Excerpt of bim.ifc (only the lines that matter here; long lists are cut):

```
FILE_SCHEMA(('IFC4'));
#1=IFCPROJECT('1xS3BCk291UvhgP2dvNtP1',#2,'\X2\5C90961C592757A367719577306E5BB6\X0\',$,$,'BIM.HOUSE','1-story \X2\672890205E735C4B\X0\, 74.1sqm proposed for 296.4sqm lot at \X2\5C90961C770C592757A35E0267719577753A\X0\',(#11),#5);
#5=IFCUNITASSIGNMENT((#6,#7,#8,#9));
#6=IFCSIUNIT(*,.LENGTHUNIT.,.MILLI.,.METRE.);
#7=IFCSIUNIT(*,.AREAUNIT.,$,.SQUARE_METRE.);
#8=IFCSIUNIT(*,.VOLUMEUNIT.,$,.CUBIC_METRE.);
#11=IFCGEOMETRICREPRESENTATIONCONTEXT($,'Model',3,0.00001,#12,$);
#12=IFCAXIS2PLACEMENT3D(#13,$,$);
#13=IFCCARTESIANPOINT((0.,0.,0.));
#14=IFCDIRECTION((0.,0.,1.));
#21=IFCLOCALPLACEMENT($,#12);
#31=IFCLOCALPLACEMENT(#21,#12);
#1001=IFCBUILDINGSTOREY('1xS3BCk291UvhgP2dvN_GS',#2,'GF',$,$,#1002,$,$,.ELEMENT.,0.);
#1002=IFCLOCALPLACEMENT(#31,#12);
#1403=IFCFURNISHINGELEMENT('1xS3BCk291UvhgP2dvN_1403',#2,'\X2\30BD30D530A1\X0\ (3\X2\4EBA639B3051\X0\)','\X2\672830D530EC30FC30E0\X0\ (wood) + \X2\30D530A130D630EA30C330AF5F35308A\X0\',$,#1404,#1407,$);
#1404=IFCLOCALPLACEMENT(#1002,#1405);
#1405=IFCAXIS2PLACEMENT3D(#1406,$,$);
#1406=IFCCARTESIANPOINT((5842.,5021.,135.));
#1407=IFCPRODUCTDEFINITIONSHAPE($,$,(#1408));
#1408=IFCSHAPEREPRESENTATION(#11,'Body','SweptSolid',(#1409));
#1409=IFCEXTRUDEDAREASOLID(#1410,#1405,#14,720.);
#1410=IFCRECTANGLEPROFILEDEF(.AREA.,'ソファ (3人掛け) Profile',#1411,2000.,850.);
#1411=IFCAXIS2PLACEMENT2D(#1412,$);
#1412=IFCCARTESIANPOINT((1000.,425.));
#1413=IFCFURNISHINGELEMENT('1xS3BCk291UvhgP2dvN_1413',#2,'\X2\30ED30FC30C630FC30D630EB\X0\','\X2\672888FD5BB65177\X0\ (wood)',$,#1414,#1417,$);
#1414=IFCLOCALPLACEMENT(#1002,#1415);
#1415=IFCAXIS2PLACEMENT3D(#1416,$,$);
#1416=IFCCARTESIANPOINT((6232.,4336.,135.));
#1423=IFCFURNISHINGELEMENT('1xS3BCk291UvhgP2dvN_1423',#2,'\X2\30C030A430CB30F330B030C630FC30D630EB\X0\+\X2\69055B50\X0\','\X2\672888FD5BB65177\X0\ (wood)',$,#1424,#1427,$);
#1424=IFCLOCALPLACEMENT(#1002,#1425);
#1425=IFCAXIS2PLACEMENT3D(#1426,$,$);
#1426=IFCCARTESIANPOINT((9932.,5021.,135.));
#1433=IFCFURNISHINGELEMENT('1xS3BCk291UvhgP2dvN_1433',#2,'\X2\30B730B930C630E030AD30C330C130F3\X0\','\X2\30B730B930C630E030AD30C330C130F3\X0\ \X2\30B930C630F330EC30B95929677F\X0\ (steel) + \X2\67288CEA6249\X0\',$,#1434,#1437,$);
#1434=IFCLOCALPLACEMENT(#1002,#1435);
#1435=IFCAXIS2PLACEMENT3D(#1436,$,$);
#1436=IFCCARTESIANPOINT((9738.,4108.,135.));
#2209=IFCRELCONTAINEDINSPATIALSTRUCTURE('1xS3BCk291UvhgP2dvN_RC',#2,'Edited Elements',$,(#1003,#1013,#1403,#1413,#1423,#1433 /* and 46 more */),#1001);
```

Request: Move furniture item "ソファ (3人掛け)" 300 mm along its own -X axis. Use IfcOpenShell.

```python
import ifcopenshell
import ifcopenshell.api.geometry
import ifcopenshell.util.placement
import ifcopenshell.util.unit

model = ifcopenshell.open("bim.ifc")
unit_scale = ifcopenshell.util.unit.calculate_unit_scale(model)

item = model.by_guid("1xS3BCk291UvhgP2dvN_1403")
matrix = ifcopenshell.util.placement.get_local_placement(item.ObjectPlacement)
matrix[:3, 3] -= matrix[:3, 0] * 0.3 / unit_scale
ifcopenshell.api.geometry.edit_object_placement(model, product=item, matrix=matrix, is_si=False)

print(ifcopenshell.util.placement.get_local_placement(item.ObjectPlacement).round(3) + 0.0)

model.write("bim-out.ifc")
```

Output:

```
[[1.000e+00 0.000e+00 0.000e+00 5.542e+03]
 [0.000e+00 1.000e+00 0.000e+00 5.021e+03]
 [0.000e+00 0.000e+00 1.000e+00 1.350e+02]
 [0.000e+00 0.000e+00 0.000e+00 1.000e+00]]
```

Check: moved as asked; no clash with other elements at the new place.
